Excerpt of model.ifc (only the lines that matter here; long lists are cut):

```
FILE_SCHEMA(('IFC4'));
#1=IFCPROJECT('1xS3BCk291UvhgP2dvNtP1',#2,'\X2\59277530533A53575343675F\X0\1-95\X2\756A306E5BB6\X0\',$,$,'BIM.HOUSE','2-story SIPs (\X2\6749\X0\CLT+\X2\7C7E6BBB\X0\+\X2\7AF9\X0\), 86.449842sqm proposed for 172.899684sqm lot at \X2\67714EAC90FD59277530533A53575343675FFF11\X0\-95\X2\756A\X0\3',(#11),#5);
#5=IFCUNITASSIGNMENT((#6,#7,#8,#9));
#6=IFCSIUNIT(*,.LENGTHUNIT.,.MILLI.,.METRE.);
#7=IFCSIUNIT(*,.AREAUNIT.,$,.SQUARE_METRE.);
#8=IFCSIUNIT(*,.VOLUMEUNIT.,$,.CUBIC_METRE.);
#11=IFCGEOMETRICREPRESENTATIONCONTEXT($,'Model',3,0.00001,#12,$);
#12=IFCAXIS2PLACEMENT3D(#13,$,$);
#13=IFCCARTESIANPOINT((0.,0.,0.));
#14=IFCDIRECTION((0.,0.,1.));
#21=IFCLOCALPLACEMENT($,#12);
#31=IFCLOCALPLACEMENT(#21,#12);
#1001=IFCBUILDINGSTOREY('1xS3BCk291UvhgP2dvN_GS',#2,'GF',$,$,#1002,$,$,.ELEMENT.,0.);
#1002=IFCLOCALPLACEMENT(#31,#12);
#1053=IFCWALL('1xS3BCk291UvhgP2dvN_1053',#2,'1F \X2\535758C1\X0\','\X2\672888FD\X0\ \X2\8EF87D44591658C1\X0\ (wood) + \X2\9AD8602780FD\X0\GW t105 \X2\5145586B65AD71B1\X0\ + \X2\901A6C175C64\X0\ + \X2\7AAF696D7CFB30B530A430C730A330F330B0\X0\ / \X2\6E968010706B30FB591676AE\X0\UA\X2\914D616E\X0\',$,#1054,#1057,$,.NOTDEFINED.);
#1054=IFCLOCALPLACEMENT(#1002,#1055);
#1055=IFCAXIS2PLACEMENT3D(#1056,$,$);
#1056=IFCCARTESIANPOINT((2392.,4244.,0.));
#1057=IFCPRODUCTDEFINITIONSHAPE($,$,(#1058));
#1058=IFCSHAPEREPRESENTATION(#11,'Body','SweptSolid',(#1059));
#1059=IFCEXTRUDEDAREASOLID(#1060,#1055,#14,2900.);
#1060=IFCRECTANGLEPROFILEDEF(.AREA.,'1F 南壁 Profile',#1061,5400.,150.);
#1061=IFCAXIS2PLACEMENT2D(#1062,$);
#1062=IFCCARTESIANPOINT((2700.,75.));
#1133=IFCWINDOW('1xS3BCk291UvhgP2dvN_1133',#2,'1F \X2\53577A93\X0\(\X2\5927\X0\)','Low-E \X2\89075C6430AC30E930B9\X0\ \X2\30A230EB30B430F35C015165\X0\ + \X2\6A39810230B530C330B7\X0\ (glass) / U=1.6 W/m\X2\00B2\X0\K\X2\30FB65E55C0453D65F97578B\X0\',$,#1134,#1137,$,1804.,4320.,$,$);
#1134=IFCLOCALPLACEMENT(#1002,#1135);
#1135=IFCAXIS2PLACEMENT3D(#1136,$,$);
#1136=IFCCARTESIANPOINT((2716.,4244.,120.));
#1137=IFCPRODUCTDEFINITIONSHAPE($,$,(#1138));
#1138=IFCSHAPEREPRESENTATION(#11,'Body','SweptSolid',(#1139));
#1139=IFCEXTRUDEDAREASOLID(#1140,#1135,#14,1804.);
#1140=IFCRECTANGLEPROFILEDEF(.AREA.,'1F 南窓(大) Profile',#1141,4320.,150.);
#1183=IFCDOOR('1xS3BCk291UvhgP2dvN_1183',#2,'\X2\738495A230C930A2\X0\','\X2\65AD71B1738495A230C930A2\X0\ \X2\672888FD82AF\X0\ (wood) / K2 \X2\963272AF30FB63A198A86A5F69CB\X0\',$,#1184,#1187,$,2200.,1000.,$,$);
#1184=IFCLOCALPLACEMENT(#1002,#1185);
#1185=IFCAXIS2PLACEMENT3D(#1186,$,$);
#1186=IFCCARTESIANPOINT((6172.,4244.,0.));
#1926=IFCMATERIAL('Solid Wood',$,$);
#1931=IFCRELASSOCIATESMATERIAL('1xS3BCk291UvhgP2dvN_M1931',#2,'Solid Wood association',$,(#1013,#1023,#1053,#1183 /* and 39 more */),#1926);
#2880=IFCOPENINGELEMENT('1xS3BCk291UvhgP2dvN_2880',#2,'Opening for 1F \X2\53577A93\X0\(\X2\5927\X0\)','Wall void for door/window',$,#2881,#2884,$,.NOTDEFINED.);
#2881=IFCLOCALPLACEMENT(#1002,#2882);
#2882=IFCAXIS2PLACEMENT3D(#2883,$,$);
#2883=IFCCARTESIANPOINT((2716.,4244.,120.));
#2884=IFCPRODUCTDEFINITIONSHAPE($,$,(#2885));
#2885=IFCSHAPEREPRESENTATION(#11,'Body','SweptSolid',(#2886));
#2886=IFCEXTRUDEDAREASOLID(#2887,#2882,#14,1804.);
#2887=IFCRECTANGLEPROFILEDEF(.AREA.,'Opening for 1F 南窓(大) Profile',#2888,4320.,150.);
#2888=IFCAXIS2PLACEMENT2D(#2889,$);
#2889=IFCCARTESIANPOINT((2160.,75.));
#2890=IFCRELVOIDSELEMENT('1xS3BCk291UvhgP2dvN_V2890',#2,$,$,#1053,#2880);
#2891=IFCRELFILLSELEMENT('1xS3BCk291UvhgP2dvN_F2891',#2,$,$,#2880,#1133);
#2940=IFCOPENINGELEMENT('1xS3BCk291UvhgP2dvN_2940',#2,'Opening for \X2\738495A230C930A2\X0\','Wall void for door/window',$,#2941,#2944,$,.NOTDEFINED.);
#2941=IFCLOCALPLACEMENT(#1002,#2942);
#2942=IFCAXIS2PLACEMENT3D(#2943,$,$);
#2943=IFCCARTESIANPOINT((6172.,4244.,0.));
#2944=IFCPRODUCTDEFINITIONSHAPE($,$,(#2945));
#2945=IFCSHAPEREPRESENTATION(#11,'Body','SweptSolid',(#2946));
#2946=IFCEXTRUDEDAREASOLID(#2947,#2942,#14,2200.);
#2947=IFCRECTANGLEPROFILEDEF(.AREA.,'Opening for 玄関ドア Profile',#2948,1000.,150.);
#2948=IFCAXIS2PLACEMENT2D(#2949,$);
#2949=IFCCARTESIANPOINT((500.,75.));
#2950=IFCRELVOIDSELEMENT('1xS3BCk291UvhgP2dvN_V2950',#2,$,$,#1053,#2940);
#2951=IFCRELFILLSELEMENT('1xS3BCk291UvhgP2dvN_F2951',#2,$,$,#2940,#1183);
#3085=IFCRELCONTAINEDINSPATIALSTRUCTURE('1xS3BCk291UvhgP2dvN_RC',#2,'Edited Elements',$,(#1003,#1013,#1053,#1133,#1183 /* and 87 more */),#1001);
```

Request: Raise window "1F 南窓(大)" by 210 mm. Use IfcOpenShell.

```python
import numpy as np
import ifcopenshell
import ifcopenshell.api.geometry
import ifcopenshell.util.placement
import ifcopenshell.util.unit

model = ifcopenshell.open("model.ifc")
unit_scale = ifcopenshell.util.unit.calculate_unit_scale(model)

window = model.by_guid("1xS3BCk291UvhgP2dvN_1133")
opening = window.FillsVoids[0].RelatingOpeningElement
dz = 0.21 / unit_scale

shift = np.array([0.0, 0.0, dz])
# The window is not placed relative to its opening, so move both.
for product in (opening, window):
    matrix = ifcopenshell.util.placement.get_local_placement(product.ObjectPlacement)
    matrix[:3, 3] += shift
    ifcopenshell.api.geometry.edit_object_placement(model, product=product, matrix=matrix, is_si=False)

print(f"moved by {dz * unit_scale:+.3f} m")

model.write("model_v2.ifc")
```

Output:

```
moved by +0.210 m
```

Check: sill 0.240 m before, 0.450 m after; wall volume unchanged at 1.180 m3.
